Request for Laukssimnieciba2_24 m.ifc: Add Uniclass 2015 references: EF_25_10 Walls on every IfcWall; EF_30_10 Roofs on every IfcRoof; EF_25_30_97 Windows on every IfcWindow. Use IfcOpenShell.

First a look at what the model holds.

```python
import ifcopenshell

model = ifcopenshell.open("Laukssimnieciba2_24 m.ifc")
print(model.schema)
print("classifications:", [c.Name for c in model.by_type("IfcClassification")])
for ifc_class in ("IfcDoor", "IfcRoof", "IfcStair", "IfcWall", "IfcWindow"):
    print(ifc_class, len(model.by_type(ifc_class)))
```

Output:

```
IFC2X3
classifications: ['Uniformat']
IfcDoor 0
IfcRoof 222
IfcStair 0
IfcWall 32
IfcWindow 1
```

```python
import ifcopenshell
import ifcopenshell.api.classification

model = ifcopenshell.open("Laukssimnieciba2_24 m.ifc")

# IFC2X3 requires Source and Edition and has no link from the project to the system.
system = model.create_entity("IfcClassification", Source="NBS", Edition="2015", Name="Uniclass 2015")

codes = {
    "IfcWall": ("EF_25_10", "Walls"),
    "IfcRoof": ("EF_30_10", "Roofs"),
    "IfcWindow": ("EF_25_30_97", "Windows"),
}
for ifc_class, (code, name) in codes.items():
    products = model.by_type(ifc_class)
    ifcopenshell.api.classification.add_reference(
        model, products=products, classification=system, identification=code, name=name
    )
    print(code, len(products))

model.write("Laukssimnieciba2_24 m_updated.ifc")
```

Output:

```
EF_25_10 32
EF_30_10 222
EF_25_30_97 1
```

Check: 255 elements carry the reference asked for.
